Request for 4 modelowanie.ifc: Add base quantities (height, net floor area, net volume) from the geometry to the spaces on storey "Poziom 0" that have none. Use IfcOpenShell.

First a look at what the model holds.

```python
import ifcopenshell
import ifcopenshell.util.element
import ifcopenshell.util.unit

model = ifcopenshell.open("4 modelowanie.ifc")
print(model.schema)
for unit_type in ("LENGTHUNIT", "AREAUNIT", "VOLUMEUNIT"):
    print(unit_type, ifcopenshell.util.unit.calculate_unit_scale(model, unit_type))
storey = next(s for s in model.by_type("IfcBuildingStorey") if s.Name == "Poziom 0")
spaces = [e for e in ifcopenshell.util.element.get_decomposition(storey) if e.is_a("IfcSpace")]
for e in sorted(spaces, key=lambda e: e.id()):
    print(e.id(), e.is_a(), e.Name, list(ifcopenshell.util.element.get_psets(e, qtos_only=True)), sep=" | ")
```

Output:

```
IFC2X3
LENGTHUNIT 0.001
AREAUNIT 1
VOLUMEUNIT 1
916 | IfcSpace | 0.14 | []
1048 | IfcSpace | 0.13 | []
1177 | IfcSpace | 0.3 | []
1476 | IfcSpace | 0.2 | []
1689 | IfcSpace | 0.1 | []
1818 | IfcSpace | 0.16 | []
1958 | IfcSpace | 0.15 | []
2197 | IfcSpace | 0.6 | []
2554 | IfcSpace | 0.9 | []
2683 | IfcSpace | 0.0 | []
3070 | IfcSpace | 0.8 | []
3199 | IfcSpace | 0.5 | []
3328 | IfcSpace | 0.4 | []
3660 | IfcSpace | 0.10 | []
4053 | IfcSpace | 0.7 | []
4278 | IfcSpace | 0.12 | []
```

```python
import ifcopenshell
import ifcopenshell.api.pset
import ifcopenshell.geom
import ifcopenshell.util.element
import ifcopenshell.util.shape
import ifcopenshell.util.unit

model = ifcopenshell.open("4 modelowanie.ifc")
unit_scale = ifcopenshell.util.unit.calculate_unit_scale(model)
area_scale = ifcopenshell.util.unit.calculate_unit_scale(model, "AREAUNIT")
volume_scale = ifcopenshell.util.unit.calculate_unit_scale(model, "VOLUMEUNIT")
settings = ifcopenshell.geom.settings()

storey = next(s for s in model.by_type("IfcBuildingStorey") if s.Name == "Poziom 0")
spaces = [e for e in ifcopenshell.util.element.get_decomposition(storey) if e.is_a("IfcSpace")]

for e in sorted(spaces, key=lambda e: e.id()):
    if ifcopenshell.util.element.get_psets(e, qtos_only=True, should_inherit=False):
        continue
    # Geometry comes back in metres, in the element's own axes.
    shape = ifcopenshell.geom.create_shape(settings, e)
    values = {
        "Height": ifcopenshell.util.shape.get_z(shape.geometry) / unit_scale,
        "NetFloorArea": ifcopenshell.util.shape.get_footprint_area(shape.geometry) / area_scale,
        "NetVolume": ifcopenshell.util.shape.get_volume(shape.geometry) / volume_scale,
    }
    qto = ifcopenshell.api.pset.add_qto(model, product=e, name="BaseQuantities")
    ifcopenshell.api.pset.edit_qto(model, qto=qto, properties=values)
    print(e.id(), {k: round(v, 3) for k, v in values.items()})

model.write("4 modelowanie-out.ifc")
```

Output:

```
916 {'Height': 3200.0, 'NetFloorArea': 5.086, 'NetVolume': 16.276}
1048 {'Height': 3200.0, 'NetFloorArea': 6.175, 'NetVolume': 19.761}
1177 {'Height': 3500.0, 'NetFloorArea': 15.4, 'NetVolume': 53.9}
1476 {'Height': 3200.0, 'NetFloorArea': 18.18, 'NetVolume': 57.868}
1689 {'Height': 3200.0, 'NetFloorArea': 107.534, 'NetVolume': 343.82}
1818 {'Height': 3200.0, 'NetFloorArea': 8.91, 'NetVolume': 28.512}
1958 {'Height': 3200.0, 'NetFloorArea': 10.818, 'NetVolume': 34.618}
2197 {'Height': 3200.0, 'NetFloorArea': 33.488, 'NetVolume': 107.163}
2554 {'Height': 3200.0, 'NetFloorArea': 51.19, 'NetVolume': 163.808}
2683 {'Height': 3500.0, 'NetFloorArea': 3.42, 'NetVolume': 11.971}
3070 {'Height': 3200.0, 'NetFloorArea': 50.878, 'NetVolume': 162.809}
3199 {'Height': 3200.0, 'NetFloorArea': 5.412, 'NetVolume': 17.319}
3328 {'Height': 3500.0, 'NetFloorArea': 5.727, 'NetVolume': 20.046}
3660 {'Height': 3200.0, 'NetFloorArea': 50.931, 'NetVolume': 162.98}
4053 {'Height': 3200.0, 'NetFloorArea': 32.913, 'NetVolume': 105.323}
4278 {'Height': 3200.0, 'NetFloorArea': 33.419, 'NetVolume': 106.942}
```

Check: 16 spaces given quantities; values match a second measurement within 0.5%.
